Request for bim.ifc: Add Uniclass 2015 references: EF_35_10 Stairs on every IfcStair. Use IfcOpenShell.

First a look at what the model holds.

```python
import ifcopenshell

model = ifcopenshell.open("bim.ifc")
print(model.schema)
print("classifications:", [c.Name for c in model.by_type("IfcClassification")])
for ifc_class in ("IfcDoor", "IfcRoof", "IfcStair", "IfcWall", "IfcWindow"):
    print(ifc_class, len(model.by_type(ifc_class)))
```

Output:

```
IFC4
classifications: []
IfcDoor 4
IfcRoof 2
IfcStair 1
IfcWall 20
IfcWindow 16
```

```python
import ifcopenshell
import ifcopenshell.api.classification

model = ifcopenshell.open("bim.ifc")

system = ifcopenshell.api.classification.add_classification(model, classification="Uniclass 2015")

codes = {
    "IfcStair": ("EF_35_10", "Stairs"),
}
for ifc_class, (code, name) in codes.items():
    products = model.by_type(ifc_class)
    ifcopenshell.api.classification.add_reference(
        model, products=products, classification=system, identification=code, name=name
    )
    print(code, len(products))

model.write("bim_edited.ifc")
```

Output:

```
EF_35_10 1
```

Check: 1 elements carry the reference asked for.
